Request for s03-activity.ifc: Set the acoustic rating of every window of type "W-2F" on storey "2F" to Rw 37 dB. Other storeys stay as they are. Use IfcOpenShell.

First a look at what the model holds.

```python
import ifcopenshell
import ifcopenshell.util.element

model = ifcopenshell.open("s03-activity.ifc")
print(model.schema)
storey = next(s for s in model.by_type("IfcBuildingStorey") if s.Name == "2F")
windows = [e for e in ifcopenshell.util.element.get_decomposition(storey) if e.is_a("IfcWindow")]
seen = {}
for e in windows:
    element_type = ifcopenshell.util.element.get_type(e)
    key = (element_type.Name if element_type != e and element_type else None, ifcopenshell.util.element.get_pset(e, "Pset_WindowCommon", "AcousticRating"))
    seen[key] = seen.get(key, 0) + 1
for (name, value), count in sorted(seen.items(), key=str):
    print(count, "x", name, "|", value)
```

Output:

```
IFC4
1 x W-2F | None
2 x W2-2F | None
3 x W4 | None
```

```python
import ifcopenshell
import ifcopenshell.api.pset
import ifcopenshell.util.element

model = ifcopenshell.open("s03-activity.ifc")

storey = next(s for s in model.by_type("IfcBuildingStorey") if s.Name == "2F")
windows = [e for e in ifcopenshell.util.element.get_decomposition(storey) if e.is_a("IfcWindow")]

count = 0
for e in windows:
    element_type = ifcopenshell.util.element.get_type(e)
    if element_type in (None, e) or element_type.Name != "W-2F":
        continue
    # add_pset returns the element's existing set when there is one.
    pset = ifcopenshell.api.pset.add_pset(model, product=e, name="Pset_WindowCommon")
    ifcopenshell.api.pset.edit_pset(model, pset=pset, properties={"AcousticRating": "Rw 37 dB"})
    count += 1

print(count, "windows updated")

model.write("s03-activity_updated.ifc")
```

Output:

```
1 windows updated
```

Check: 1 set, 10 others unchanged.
